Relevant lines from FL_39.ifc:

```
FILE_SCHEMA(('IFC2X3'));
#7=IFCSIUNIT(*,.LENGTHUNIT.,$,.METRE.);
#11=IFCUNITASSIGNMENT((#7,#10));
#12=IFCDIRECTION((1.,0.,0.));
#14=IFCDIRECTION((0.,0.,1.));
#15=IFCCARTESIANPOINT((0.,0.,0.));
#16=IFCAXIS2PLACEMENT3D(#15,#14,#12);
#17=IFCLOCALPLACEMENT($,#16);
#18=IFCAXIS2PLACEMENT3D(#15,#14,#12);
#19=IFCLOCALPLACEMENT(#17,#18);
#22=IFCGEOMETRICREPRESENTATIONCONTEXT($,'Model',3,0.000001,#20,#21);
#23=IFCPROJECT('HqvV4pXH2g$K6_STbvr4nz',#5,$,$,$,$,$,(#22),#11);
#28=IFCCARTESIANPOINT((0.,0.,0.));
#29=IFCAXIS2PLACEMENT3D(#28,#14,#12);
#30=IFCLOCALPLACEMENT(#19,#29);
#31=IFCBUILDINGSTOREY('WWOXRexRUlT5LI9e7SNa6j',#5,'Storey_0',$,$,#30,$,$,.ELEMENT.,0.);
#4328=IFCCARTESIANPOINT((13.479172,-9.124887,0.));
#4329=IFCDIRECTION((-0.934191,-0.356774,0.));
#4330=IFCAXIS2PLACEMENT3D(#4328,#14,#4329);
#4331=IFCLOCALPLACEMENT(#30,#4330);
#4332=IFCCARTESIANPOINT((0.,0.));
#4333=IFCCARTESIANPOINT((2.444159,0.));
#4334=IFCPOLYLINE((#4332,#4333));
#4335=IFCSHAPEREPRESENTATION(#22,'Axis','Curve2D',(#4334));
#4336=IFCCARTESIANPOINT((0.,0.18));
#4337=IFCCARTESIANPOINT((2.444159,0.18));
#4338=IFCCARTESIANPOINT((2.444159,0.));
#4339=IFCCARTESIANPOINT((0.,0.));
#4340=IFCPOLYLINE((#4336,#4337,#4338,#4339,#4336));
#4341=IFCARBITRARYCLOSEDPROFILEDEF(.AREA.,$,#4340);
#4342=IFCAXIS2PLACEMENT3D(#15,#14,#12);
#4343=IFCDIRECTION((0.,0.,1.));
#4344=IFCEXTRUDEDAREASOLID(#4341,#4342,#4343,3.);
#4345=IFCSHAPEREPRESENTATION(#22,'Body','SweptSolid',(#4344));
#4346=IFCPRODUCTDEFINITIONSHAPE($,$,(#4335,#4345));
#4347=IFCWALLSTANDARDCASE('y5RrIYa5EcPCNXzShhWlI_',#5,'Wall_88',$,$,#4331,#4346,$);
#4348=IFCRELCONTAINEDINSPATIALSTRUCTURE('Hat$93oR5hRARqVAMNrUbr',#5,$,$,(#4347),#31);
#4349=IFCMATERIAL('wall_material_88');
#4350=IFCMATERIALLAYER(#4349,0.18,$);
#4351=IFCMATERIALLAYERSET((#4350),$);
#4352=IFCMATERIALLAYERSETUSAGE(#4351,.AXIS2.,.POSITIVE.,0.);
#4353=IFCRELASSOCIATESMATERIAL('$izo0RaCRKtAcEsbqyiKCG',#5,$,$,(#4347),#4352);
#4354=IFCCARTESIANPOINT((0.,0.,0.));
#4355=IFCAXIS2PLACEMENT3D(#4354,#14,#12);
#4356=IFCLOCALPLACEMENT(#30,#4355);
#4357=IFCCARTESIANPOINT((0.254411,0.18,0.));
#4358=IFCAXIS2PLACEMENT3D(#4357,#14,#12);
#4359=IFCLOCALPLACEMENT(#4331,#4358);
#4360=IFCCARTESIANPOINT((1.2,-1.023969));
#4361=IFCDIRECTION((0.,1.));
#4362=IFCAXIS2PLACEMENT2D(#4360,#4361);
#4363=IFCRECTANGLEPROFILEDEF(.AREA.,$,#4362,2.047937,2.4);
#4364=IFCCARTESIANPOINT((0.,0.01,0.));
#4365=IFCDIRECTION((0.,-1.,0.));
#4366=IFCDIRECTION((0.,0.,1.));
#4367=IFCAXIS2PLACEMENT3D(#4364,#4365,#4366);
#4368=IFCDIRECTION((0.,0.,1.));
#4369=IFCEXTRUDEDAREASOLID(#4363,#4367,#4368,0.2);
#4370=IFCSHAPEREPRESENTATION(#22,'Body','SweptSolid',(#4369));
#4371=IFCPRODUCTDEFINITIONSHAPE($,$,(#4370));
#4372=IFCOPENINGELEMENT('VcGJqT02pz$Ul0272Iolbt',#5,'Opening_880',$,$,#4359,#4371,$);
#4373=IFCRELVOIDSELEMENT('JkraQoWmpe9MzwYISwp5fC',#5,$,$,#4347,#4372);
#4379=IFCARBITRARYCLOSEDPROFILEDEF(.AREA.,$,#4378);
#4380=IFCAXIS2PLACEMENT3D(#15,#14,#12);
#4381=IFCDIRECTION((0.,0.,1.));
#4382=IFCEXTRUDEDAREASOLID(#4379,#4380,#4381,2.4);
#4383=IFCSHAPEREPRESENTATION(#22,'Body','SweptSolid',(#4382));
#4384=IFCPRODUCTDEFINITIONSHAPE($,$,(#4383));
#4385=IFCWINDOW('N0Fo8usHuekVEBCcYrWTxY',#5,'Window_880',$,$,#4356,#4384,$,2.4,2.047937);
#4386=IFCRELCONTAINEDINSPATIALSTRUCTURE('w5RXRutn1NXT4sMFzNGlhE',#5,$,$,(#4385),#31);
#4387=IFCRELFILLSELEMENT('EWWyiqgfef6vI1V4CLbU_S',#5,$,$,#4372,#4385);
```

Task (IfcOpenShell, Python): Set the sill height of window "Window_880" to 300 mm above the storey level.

```python
import numpy as np
import ifcopenshell
import ifcopenshell.api.geometry
import ifcopenshell.geom
import ifcopenshell.util.element
import ifcopenshell.util.placement
import ifcopenshell.util.shape
import ifcopenshell.util.unit

model = ifcopenshell.open("FL_39.ifc")
unit_scale = ifcopenshell.util.unit.calculate_unit_scale(model)

window = model.by_id(4385)
opening = window.FillsVoids[0].RelatingOpeningElement
storey = ifcopenshell.util.element.get_container(window, ifc_class="IfcBuildingStorey")
level = ifcopenshell.util.placement.get_local_placement(storey.ObjectPlacement)[2, 3]

# The opening's origin need not be at the sill, so measure its lowest point.
shape = ifcopenshell.geom.create_shape(ifcopenshell.geom.settings(), opening)
bottom = ifcopenshell.util.shape.get_shape_bottom_elevation(shape, shape.geometry) / unit_scale
dz = level + 0.3 - bottom

shift = np.array([0.0, 0.0, dz])
# The window is not placed relative to its opening, so move both.
for product in (opening, window):
    matrix = ifcopenshell.util.placement.get_local_placement(product.ObjectPlacement)
    matrix[:3, 3] += shift
    ifcopenshell.api.geometry.edit_object_placement(model, product=product, matrix=matrix, is_si=False)

print(f"moved by {dz * unit_scale:+.3f} m")

model.write("FL_39-out.ifc")
```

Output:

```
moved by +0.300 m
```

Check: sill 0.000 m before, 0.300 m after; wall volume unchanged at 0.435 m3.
